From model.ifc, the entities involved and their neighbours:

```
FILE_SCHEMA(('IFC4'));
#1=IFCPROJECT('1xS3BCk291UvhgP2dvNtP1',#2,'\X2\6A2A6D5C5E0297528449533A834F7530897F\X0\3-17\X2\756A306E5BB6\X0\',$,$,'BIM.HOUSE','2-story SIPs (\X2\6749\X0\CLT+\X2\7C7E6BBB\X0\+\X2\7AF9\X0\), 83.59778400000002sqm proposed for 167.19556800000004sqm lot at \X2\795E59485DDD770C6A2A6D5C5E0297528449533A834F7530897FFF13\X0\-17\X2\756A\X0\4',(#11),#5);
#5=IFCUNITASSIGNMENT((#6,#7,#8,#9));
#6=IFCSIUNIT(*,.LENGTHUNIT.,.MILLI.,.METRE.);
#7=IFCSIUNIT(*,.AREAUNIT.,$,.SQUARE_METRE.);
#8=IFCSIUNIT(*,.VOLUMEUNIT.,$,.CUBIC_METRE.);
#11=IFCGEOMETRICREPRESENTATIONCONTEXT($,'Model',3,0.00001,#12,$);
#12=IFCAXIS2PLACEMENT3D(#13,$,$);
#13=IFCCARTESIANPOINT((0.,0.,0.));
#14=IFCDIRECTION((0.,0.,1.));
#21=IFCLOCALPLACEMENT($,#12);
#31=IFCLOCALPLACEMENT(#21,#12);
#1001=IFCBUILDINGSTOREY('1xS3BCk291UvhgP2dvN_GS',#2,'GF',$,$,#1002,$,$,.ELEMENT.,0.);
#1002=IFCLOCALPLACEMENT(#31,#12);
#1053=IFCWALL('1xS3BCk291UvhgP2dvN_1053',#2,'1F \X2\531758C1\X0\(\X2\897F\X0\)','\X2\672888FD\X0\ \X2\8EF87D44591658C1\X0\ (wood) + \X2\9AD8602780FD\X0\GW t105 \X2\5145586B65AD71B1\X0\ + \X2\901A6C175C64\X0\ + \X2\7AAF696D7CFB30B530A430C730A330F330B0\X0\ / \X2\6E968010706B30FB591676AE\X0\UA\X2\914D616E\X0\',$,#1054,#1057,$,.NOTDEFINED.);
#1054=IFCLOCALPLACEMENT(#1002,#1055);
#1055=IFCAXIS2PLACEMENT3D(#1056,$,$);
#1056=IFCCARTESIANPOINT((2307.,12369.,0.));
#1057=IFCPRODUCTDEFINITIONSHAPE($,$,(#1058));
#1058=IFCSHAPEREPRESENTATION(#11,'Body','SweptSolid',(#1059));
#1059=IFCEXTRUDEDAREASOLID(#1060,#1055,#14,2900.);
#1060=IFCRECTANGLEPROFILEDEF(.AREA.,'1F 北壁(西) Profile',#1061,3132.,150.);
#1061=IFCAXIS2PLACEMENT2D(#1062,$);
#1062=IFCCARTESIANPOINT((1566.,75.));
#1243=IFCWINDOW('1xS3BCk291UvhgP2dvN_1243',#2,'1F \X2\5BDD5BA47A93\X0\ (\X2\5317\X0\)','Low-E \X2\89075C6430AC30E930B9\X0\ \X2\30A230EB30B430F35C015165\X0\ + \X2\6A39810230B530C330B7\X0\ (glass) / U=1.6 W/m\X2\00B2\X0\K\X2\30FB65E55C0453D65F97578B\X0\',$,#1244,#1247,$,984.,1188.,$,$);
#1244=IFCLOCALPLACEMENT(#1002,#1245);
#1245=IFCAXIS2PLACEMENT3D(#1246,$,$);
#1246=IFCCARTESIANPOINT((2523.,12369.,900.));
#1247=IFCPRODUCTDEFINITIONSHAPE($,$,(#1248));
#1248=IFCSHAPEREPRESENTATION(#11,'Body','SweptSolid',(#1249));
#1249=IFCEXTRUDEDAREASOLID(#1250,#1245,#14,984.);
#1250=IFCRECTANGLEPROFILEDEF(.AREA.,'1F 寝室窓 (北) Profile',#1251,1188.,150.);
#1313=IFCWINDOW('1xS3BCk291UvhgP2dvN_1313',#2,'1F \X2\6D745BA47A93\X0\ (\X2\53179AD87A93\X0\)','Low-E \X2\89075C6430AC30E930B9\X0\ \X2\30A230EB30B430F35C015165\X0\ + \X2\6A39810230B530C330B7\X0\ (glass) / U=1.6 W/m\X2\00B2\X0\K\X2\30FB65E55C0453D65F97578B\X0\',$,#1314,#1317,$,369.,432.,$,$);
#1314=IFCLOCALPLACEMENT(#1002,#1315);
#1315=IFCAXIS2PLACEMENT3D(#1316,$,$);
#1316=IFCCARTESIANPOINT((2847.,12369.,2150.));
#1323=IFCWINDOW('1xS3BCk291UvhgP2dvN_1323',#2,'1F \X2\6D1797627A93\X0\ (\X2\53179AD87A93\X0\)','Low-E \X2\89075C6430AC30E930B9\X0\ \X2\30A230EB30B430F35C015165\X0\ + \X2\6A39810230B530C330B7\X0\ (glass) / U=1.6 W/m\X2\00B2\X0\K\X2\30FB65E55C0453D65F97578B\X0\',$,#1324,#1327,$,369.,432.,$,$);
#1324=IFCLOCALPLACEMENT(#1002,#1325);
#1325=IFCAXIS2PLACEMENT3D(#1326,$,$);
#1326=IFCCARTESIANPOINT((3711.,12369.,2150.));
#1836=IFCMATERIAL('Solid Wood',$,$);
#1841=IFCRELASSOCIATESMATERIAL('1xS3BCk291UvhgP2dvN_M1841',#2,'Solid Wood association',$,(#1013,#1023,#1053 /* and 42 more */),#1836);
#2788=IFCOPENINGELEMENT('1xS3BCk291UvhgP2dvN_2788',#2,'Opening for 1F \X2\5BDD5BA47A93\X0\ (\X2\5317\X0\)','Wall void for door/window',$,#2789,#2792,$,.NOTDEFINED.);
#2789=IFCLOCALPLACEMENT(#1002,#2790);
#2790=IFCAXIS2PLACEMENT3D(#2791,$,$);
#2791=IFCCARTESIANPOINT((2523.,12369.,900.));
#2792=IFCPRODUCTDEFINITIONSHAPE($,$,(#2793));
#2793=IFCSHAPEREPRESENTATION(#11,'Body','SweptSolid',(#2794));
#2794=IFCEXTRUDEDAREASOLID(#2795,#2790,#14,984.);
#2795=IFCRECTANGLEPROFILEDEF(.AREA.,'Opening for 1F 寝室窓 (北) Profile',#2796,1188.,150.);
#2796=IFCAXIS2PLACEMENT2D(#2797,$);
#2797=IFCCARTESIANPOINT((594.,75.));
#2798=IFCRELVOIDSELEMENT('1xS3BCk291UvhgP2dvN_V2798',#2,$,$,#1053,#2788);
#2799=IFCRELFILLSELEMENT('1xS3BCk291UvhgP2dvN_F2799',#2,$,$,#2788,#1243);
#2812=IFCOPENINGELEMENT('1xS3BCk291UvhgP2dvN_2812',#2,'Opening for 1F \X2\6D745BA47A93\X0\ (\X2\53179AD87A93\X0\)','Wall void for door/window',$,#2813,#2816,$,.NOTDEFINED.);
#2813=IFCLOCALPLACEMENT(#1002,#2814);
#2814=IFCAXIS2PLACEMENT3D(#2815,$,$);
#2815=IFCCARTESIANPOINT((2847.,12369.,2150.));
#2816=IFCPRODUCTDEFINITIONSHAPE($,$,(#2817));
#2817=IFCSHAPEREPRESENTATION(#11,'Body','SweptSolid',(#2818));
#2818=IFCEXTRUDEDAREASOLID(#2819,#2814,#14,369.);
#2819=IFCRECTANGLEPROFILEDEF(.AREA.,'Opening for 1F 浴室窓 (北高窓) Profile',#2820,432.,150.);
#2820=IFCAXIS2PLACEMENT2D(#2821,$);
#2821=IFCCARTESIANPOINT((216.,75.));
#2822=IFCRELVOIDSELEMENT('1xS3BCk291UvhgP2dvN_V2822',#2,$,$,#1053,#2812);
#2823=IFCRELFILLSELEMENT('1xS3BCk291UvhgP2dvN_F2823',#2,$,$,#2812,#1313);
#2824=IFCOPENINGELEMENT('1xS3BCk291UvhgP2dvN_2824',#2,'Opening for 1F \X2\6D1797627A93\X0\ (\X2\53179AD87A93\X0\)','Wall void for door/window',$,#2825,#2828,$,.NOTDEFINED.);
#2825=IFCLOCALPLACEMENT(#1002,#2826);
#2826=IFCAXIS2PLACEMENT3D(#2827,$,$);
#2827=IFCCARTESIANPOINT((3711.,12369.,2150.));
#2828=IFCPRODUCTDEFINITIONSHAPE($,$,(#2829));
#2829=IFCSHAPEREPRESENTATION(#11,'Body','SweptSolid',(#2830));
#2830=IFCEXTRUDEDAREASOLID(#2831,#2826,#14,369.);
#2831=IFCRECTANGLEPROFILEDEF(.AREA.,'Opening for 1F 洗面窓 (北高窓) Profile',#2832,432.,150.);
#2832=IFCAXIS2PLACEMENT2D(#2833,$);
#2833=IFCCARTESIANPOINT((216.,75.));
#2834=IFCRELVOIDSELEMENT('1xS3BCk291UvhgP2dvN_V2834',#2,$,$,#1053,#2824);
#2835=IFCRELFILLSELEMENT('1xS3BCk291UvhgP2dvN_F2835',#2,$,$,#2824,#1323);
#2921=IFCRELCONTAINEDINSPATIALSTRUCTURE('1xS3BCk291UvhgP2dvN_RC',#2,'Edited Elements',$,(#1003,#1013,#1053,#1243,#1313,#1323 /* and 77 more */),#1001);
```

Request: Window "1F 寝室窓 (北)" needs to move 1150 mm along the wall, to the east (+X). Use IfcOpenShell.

```python
import ifcopenshell
import ifcopenshell.api.geometry
import ifcopenshell.util.placement

model = ifcopenshell.open("model.ifc")

window = model.by_id(1243)
opening = window.FillsVoids[0].RelatingOpeningElement
wall = opening.VoidsElements[0].RelatingBuildingElement

wall_matrix = ifcopenshell.util.placement.get_local_placement(wall.ObjectPlacement)
shift = wall_matrix[:3, 0] * 1150.0
before = ifcopenshell.util.placement.get_local_placement(window.ObjectPlacement)[:3, 3].copy()

# The window is not placed relative to its opening, so move both.
for product in (opening, window):
    matrix = ifcopenshell.util.placement.get_local_placement(product.ObjectPlacement)
    matrix[:3, 3] += shift
    ifcopenshell.api.geometry.edit_object_placement(model, product=product, matrix=matrix, is_si=False)

after = ifcopenshell.util.placement.get_local_placement(window.ObjectPlacement)[:3, 3]
print("window moved by", (after - before).round(3) + 0.0)

model.write("model_edited.ifc")
```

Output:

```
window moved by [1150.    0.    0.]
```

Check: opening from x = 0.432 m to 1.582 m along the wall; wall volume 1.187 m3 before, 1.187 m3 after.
